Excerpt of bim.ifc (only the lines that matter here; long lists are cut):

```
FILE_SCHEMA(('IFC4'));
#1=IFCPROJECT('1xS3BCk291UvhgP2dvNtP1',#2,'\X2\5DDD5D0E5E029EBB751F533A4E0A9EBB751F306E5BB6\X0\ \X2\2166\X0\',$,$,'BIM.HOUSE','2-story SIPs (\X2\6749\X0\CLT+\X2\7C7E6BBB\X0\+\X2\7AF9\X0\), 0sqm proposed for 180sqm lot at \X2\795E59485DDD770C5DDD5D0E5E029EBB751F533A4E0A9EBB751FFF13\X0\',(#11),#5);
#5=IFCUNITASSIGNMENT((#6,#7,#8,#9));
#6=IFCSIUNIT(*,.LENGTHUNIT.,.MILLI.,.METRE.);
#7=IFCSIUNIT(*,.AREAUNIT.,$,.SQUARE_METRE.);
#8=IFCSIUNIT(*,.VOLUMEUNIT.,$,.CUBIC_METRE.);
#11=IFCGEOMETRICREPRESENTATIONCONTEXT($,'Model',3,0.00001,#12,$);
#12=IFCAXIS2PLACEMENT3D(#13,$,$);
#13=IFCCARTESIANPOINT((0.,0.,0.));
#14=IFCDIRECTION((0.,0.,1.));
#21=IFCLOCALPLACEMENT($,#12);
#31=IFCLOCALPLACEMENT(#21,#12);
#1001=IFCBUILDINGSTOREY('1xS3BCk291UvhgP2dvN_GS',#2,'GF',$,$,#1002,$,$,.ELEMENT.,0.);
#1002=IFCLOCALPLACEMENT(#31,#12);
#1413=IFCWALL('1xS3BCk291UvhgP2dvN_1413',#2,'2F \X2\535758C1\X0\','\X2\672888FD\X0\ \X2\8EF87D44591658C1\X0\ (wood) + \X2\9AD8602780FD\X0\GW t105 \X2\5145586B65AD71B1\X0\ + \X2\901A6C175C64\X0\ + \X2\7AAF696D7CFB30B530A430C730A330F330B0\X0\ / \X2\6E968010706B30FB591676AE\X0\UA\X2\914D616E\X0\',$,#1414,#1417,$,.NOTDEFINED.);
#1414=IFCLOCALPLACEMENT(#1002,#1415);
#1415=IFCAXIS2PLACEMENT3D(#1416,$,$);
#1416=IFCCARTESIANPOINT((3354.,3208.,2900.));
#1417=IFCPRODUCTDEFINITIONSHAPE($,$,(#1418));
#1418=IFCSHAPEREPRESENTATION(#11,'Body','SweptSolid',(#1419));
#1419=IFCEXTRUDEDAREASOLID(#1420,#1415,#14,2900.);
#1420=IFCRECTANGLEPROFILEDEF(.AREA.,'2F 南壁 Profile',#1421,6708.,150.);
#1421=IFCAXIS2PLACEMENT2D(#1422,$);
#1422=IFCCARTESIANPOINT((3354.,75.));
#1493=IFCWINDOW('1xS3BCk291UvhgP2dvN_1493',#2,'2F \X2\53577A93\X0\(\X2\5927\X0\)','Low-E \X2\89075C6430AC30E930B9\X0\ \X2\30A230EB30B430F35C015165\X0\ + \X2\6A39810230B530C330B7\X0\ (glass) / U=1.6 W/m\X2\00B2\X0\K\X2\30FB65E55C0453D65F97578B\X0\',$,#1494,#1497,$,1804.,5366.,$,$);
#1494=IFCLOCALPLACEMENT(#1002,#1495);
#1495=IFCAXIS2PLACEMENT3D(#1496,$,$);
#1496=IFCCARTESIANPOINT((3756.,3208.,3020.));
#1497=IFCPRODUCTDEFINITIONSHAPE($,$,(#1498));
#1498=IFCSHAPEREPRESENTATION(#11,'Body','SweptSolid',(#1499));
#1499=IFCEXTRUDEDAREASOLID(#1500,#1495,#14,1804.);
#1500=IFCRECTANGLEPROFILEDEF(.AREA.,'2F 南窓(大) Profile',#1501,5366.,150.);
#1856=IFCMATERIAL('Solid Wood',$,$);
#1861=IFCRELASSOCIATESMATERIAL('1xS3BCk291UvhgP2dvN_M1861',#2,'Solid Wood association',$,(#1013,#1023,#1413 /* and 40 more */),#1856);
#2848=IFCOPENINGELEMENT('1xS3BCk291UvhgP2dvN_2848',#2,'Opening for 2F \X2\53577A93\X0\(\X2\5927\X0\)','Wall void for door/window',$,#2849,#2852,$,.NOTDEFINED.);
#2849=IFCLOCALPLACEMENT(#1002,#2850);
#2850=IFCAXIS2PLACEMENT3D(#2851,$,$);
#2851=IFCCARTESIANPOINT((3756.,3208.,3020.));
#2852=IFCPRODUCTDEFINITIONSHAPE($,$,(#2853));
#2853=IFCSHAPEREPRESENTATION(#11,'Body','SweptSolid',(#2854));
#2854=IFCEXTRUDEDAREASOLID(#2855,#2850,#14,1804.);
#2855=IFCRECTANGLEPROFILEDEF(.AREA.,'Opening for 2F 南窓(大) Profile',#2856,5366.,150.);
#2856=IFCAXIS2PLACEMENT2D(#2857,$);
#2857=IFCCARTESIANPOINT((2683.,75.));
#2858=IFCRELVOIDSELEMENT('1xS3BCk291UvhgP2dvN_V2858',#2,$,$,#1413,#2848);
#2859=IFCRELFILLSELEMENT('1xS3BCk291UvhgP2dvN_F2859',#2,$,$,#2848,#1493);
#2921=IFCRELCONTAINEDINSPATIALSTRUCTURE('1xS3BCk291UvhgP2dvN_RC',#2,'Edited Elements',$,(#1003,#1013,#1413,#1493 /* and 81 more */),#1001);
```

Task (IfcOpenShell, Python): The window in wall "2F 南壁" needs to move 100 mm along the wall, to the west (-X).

```python
import ifcopenshell
import ifcopenshell.api.geometry
import ifcopenshell.util.placement
import ifcopenshell.util.unit

model = ifcopenshell.open("bim.ifc")
unit_scale = ifcopenshell.util.unit.calculate_unit_scale(model)

window = model.by_guid("1xS3BCk291UvhgP2dvN_1493")
opening = window.FillsVoids[0].RelatingOpeningElement
wall = opening.VoidsElements[0].RelatingBuildingElement

wall_matrix = ifcopenshell.util.placement.get_local_placement(wall.ObjectPlacement)
shift = wall_matrix[:3, 0] * -0.1 / unit_scale
before = ifcopenshell.util.placement.get_local_placement(window.ObjectPlacement)[:3, 3].copy()

# The window is not placed relative to its opening, so move both.
for product in (opening, window):
    matrix = ifcopenshell.util.placement.get_local_placement(product.ObjectPlacement)
    matrix[:3, 3] += shift
    ifcopenshell.api.geometry.edit_object_placement(model, product=product, matrix=matrix, is_si=False)

after = ifcopenshell.util.placement.get_local_placement(window.ObjectPlacement)[:3, 3]
print("window moved by", (after - before).round(3) + 0.0)

model.write("bim_rev.ifc")
```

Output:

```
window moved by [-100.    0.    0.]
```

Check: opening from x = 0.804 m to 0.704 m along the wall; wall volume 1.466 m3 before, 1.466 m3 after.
